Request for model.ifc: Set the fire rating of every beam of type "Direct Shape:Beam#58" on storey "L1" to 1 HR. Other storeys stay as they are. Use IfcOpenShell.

First a look at what the model holds.

```python
import ifcopenshell
import ifcopenshell.util.element

model = ifcopenshell.open("model.ifc")
print(model.schema)
storey = next(s for s in model.by_type("IfcBuildingStorey") if s.Name == "L1")
beams = [e for e in ifcopenshell.util.element.get_decomposition(storey) if e.is_a("IfcBeam")]
seen = {}
for e in beams:
    element_type = ifcopenshell.util.element.get_type(e)
    key = (element_type.Name if element_type != e and element_type else None, ifcopenshell.util.element.get_pset(e, "Pset_BeamCommon", "FireRating"))
    seen[key] = seen.get(key, 0) + 1
for (name, value), count in sorted(seen.items(), key=str):
    print(count, "x", name, "|", value)
```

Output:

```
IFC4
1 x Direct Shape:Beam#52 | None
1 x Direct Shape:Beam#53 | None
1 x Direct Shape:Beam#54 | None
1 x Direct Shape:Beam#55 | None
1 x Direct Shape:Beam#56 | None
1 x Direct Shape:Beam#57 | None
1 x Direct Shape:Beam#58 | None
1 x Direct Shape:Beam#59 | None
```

```python
import ifcopenshell
import ifcopenshell.api.pset
import ifcopenshell.util.element

model = ifcopenshell.open("model.ifc")

storey = next(s for s in model.by_type("IfcBuildingStorey") if s.Name == "L1")
beams = [e for e in ifcopenshell.util.element.get_decomposition(storey) if e.is_a("IfcBeam")]

count = 0
for e in beams:
    element_type = ifcopenshell.util.element.get_type(e)
    if element_type in (None, e) or element_type.Name != "Direct Shape:Beam#58":
        continue
    # add_pset returns the element's existing set when there is one.
    pset = ifcopenshell.api.pset.add_pset(model, product=e, name="Pset_BeamCommon")
    ifcopenshell.api.pset.edit_pset(model, pset=pset, properties={"FireRating": "1 HR"})
    count += 1

print(count, "beams updated")

model.write("model_rev.ifc")
```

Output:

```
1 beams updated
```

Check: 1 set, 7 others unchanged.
